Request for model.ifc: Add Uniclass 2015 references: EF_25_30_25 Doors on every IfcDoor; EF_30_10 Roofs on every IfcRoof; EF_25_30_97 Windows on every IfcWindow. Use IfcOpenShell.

First a look at what the model holds.

```python
import ifcopenshell

model = ifcopenshell.open("model.ifc")
print(model.schema)
print("classifications:", [c.Name for c in model.by_type("IfcClassification")])
for ifc_class in ("IfcDoor", "IfcRoof", "IfcStair", "IfcWall", "IfcWindow"):
    print(ifc_class, len(model.by_type(ifc_class)))
```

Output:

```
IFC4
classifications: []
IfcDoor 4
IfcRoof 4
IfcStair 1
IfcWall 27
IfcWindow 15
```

```python
import ifcopenshell
import ifcopenshell.api.classification

model = ifcopenshell.open("model.ifc")

system = ifcopenshell.api.classification.add_classification(model, classification="Uniclass 2015")

codes = {
    "IfcDoor": ("EF_25_30_25", "Doors"),
    "IfcRoof": ("EF_30_10", "Roofs"),
    "IfcWindow": ("EF_25_30_97", "Windows"),
}
for ifc_class, (code, name) in codes.items():
    products = model.by_type(ifc_class)
    ifcopenshell.api.classification.add_reference(
        model, products=products, classification=system, identification=code, name=name
    )
    print(code, len(products))

model.write("model_updated.ifc")
```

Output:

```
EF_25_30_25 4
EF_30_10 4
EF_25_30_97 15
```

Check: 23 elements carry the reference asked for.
